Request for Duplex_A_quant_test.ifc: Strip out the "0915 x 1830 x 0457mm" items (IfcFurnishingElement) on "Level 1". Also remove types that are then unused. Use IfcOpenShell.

First a look at what the model holds.

```python
import ifcopenshell
import ifcopenshell.util.element

model = ifcopenshell.open("Duplex_A_quant_test.ifc")
print(model.schema)
storey = next(s for s in model.by_type("IfcBuildingStorey") if s.Name == "Level 1")
furniture = [e for e in ifcopenshell.util.element.get_decomposition(storey) if e.is_a("IfcFurnishingElement")]
seen = {}
for e in furniture:
    element_type = ifcopenshell.util.element.get_type(e)
    name = element_type.Name if element_type not in (None, e) else None
    seen[name] = seen.get(name, 0) + 1
for name, count in sorted(seen.items(), key=str):
    print(count, "x", name)
```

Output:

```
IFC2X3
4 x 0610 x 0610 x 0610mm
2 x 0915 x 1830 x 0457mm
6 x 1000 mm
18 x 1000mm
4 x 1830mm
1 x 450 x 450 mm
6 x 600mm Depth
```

```python
import ifcopenshell
import ifcopenshell.api.root
import ifcopenshell.util.element

model = ifcopenshell.open("Duplex_A_quant_test.ifc")

storey = next(s for s in model.by_type("IfcBuildingStorey") if s.Name == "Level 1")
furniture = [e for e in ifcopenshell.util.element.get_decomposition(storey) if e.is_a("IfcFurnishingElement")]
targets = [e for e in furniture if (t := ifcopenshell.util.element.get_type(e)) not in (None, e) and t.Name == "0915 x 1830 x 0457mm"]
types = {ifcopenshell.util.element.get_type(e) for e in targets} - {None, *targets}

for e in targets:
    ifcopenshell.api.root.remove_product(model, product=e)
print(len(targets), "removed")

unused = [t for t in types if not ifcopenshell.util.element.get_types(t)]
for t in unused:
    ifcopenshell.api.root.remove_product(model, product=t)
print(len(unused), "unused types removed")

model.write("Duplex_A_quant_test_updated.ifc")
```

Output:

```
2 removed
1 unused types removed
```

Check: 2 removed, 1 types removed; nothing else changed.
